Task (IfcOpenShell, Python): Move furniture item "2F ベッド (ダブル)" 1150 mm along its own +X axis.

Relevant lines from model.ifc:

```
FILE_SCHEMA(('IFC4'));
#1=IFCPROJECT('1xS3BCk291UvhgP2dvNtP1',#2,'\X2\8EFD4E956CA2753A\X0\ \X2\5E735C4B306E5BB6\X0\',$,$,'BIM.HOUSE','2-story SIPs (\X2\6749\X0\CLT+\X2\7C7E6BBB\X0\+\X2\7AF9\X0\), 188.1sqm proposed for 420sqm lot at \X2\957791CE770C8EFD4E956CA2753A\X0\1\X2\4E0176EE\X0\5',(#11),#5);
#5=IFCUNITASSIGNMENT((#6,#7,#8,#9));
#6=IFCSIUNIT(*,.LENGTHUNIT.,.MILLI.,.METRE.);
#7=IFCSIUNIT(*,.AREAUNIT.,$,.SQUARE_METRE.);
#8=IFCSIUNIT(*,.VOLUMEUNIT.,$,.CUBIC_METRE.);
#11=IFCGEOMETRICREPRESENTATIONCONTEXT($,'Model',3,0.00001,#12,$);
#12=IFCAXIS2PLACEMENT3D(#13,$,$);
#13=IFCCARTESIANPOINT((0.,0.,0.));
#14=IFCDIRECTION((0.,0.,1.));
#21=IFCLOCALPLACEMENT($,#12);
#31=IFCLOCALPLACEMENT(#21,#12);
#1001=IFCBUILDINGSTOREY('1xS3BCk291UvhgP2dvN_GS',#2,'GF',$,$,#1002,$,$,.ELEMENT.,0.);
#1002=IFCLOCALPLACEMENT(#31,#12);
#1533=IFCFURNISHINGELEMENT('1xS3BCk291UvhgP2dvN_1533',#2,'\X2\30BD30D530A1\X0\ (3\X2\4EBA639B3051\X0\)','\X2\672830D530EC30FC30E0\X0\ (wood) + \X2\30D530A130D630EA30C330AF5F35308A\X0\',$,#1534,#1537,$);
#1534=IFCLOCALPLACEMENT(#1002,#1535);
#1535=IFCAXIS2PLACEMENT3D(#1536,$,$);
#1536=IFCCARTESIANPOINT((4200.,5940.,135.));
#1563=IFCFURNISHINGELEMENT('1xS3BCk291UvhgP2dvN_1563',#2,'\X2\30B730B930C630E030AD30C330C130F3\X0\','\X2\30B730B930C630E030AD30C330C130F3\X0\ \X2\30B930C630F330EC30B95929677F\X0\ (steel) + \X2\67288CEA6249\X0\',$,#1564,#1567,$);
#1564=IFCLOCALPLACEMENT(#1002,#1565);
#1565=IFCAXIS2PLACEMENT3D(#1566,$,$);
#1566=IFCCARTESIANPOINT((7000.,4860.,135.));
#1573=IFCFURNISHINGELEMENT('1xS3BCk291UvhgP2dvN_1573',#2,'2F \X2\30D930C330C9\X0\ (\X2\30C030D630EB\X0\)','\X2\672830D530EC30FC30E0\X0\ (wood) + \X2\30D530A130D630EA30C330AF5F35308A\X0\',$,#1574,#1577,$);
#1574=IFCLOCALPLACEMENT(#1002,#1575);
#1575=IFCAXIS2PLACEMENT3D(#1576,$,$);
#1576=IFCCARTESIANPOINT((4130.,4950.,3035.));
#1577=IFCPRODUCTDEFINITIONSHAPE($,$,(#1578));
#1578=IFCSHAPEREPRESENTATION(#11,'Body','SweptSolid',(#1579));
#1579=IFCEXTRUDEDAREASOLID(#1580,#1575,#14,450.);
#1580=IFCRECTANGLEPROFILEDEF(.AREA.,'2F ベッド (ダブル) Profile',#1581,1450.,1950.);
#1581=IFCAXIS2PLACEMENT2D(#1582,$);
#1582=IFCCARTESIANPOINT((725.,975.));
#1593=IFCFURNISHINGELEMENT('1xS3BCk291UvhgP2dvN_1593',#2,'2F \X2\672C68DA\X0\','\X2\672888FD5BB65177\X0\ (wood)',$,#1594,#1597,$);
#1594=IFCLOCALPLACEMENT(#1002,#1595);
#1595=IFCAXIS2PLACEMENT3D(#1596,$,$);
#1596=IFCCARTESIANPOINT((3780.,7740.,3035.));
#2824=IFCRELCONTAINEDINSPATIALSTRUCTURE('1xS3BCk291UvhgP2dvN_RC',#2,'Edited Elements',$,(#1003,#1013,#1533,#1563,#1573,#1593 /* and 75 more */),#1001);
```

```python
import ifcopenshell
import ifcopenshell.api.geometry
import ifcopenshell.util.placement
import ifcopenshell.util.unit

model = ifcopenshell.open("model.ifc")
unit_scale = ifcopenshell.util.unit.calculate_unit_scale(model)

item = model.by_guid("1xS3BCk291UvhgP2dvN_1573")
matrix = ifcopenshell.util.placement.get_local_placement(item.ObjectPlacement)
matrix[:3, 3] += matrix[:3, 0] * 1.15 / unit_scale
ifcopenshell.api.geometry.edit_object_placement(model, product=item, matrix=matrix, is_si=False)

print(ifcopenshell.util.placement.get_local_placement(item.ObjectPlacement).round(3) + 0.0)

model.write("model_edited.ifc")
```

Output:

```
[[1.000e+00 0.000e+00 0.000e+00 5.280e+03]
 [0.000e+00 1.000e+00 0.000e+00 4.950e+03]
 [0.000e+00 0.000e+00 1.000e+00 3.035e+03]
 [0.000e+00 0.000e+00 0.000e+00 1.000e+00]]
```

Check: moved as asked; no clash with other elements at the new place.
